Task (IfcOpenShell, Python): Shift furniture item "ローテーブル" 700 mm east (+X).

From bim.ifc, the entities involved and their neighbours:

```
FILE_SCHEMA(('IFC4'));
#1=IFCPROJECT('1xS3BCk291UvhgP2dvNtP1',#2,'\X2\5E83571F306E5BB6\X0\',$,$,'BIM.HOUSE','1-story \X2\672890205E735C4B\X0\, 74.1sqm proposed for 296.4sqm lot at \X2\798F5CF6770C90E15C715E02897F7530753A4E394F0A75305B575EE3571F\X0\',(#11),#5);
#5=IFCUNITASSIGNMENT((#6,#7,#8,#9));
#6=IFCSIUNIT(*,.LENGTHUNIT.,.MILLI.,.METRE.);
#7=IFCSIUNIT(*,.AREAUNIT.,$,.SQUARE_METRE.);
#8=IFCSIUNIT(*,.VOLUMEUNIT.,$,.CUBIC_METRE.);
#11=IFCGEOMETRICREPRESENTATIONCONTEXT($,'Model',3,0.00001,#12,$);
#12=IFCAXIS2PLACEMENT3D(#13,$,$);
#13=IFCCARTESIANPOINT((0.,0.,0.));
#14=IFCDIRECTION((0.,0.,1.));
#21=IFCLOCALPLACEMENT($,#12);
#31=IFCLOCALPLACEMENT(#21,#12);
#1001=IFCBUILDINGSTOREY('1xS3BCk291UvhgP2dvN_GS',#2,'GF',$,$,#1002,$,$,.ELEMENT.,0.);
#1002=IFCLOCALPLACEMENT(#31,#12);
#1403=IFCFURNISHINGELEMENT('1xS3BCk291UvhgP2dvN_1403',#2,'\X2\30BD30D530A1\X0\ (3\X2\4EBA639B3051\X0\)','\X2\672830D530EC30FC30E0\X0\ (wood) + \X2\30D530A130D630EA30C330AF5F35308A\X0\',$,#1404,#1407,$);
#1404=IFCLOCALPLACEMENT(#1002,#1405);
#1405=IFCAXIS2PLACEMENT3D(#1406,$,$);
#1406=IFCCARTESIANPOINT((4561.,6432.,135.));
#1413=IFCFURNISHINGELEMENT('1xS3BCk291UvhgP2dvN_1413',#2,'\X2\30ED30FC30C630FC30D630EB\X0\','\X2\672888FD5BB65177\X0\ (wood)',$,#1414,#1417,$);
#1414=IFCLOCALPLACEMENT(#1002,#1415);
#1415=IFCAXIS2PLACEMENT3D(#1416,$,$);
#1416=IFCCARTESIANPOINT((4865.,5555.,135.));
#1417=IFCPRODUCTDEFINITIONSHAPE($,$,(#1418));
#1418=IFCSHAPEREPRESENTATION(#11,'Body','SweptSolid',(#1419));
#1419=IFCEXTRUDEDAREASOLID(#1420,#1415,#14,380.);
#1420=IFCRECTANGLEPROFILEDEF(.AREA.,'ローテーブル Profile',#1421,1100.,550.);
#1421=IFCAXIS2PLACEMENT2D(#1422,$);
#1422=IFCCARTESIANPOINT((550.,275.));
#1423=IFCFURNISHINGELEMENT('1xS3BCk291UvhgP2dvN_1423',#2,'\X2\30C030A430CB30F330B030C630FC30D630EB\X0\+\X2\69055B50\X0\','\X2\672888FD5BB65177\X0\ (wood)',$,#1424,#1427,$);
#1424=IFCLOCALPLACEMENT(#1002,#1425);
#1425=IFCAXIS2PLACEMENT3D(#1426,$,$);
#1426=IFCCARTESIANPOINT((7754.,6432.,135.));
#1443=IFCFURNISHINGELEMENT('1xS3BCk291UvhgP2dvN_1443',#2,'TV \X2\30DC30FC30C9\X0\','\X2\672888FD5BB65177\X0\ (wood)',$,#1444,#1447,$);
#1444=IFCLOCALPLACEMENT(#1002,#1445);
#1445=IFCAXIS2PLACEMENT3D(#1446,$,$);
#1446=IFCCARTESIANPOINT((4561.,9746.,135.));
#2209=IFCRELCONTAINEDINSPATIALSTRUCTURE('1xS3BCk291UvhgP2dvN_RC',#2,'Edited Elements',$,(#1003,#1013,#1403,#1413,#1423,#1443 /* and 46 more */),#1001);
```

```python
import ifcopenshell
import ifcopenshell.api.geometry
import ifcopenshell.util.placement
import ifcopenshell.util.unit

model = ifcopenshell.open("bim.ifc")
unit_scale = ifcopenshell.util.unit.calculate_unit_scale(model)

item = model.by_id(1413)
matrix = ifcopenshell.util.placement.get_local_placement(item.ObjectPlacement)
matrix[0, 3] += 0.7 / unit_scale
ifcopenshell.api.geometry.edit_object_placement(model, product=item, matrix=matrix, is_si=False)

print(ifcopenshell.util.placement.get_local_placement(item.ObjectPlacement).round(3) + 0.0)

model.write("bim_updated.ifc")
```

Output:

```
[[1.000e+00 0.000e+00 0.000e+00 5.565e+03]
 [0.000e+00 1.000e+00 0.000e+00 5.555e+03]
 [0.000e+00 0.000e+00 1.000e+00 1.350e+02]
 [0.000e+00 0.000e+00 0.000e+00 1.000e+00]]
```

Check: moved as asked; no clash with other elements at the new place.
